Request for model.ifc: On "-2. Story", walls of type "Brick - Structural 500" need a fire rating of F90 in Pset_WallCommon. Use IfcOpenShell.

First a look at what the model holds.

```python
import ifcopenshell
import ifcopenshell.util.element

model = ifcopenshell.open("model.ifc")
print(model.schema)
storey = next(s for s in model.by_type("IfcBuildingStorey") if s.Name == "-2. Story")
walls = [e for e in ifcopenshell.util.element.get_decomposition(storey) if e.is_a("IfcWall")]
seen = {}
for e in walls:
    element_type = ifcopenshell.util.element.get_type(e)
    key = (element_type.Name if element_type != e and element_type else None, ifcopenshell.util.element.get_pset(e, "Pset_WallCommon", "FireRating"))
    seen[key] = seen.get(key, 0) + 1
for (name, value), count in sorted(seen.items(), key=str):
    print(count, "x", name, "|", value)
```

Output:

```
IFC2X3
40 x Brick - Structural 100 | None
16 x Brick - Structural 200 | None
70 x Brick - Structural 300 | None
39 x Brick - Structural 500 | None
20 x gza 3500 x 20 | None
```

```python
import ifcopenshell
import ifcopenshell.api.pset
import ifcopenshell.util.element

model = ifcopenshell.open("model.ifc")

storey = next(s for s in model.by_type("IfcBuildingStorey") if s.Name == "-2. Story")
walls = [e for e in ifcopenshell.util.element.get_decomposition(storey) if e.is_a("IfcWall")]

count = 0
for e in walls:
    element_type = ifcopenshell.util.element.get_type(e)
    if element_type in (None, e) or element_type.Name != "Brick - Structural 500":
        continue
    # add_pset returns the element's existing set when there is one.
    pset = ifcopenshell.api.pset.add_pset(model, product=e, name="Pset_WallCommon")
    ifcopenshell.api.pset.edit_pset(model, pset=pset, properties={"FireRating": "F90"})
    count += 1

print(count, "walls updated")

model.write("model_rev.ifc")
```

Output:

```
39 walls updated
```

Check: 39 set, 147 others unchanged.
